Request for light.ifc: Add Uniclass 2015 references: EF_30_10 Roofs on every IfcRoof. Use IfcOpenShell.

First a look at what the model holds.

```python
import ifcopenshell

model = ifcopenshell.open("light.ifc")
print(model.schema)
print("classifications:", [c.Name for c in model.by_type("IfcClassification")])
for ifc_class in ("IfcDoor", "IfcRoof", "IfcStair", "IfcWall", "IfcWindow"):
    print(ifc_class, len(model.by_type(ifc_class)))
```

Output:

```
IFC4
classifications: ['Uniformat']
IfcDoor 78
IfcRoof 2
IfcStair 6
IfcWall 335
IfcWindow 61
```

```python
import ifcopenshell
import ifcopenshell.api.classification

model = ifcopenshell.open("light.ifc")

system = ifcopenshell.api.classification.add_classification(model, classification="Uniclass 2015")

codes = {
    "IfcRoof": ("EF_30_10", "Roofs"),
}
for ifc_class, (code, name) in codes.items():
    products = model.by_type(ifc_class)
    ifcopenshell.api.classification.add_reference(
        model, products=products, classification=system, identification=code, name=name
    )
    print(code, len(products))

model.write("light_v2.ifc")
```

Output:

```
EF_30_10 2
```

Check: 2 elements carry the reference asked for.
